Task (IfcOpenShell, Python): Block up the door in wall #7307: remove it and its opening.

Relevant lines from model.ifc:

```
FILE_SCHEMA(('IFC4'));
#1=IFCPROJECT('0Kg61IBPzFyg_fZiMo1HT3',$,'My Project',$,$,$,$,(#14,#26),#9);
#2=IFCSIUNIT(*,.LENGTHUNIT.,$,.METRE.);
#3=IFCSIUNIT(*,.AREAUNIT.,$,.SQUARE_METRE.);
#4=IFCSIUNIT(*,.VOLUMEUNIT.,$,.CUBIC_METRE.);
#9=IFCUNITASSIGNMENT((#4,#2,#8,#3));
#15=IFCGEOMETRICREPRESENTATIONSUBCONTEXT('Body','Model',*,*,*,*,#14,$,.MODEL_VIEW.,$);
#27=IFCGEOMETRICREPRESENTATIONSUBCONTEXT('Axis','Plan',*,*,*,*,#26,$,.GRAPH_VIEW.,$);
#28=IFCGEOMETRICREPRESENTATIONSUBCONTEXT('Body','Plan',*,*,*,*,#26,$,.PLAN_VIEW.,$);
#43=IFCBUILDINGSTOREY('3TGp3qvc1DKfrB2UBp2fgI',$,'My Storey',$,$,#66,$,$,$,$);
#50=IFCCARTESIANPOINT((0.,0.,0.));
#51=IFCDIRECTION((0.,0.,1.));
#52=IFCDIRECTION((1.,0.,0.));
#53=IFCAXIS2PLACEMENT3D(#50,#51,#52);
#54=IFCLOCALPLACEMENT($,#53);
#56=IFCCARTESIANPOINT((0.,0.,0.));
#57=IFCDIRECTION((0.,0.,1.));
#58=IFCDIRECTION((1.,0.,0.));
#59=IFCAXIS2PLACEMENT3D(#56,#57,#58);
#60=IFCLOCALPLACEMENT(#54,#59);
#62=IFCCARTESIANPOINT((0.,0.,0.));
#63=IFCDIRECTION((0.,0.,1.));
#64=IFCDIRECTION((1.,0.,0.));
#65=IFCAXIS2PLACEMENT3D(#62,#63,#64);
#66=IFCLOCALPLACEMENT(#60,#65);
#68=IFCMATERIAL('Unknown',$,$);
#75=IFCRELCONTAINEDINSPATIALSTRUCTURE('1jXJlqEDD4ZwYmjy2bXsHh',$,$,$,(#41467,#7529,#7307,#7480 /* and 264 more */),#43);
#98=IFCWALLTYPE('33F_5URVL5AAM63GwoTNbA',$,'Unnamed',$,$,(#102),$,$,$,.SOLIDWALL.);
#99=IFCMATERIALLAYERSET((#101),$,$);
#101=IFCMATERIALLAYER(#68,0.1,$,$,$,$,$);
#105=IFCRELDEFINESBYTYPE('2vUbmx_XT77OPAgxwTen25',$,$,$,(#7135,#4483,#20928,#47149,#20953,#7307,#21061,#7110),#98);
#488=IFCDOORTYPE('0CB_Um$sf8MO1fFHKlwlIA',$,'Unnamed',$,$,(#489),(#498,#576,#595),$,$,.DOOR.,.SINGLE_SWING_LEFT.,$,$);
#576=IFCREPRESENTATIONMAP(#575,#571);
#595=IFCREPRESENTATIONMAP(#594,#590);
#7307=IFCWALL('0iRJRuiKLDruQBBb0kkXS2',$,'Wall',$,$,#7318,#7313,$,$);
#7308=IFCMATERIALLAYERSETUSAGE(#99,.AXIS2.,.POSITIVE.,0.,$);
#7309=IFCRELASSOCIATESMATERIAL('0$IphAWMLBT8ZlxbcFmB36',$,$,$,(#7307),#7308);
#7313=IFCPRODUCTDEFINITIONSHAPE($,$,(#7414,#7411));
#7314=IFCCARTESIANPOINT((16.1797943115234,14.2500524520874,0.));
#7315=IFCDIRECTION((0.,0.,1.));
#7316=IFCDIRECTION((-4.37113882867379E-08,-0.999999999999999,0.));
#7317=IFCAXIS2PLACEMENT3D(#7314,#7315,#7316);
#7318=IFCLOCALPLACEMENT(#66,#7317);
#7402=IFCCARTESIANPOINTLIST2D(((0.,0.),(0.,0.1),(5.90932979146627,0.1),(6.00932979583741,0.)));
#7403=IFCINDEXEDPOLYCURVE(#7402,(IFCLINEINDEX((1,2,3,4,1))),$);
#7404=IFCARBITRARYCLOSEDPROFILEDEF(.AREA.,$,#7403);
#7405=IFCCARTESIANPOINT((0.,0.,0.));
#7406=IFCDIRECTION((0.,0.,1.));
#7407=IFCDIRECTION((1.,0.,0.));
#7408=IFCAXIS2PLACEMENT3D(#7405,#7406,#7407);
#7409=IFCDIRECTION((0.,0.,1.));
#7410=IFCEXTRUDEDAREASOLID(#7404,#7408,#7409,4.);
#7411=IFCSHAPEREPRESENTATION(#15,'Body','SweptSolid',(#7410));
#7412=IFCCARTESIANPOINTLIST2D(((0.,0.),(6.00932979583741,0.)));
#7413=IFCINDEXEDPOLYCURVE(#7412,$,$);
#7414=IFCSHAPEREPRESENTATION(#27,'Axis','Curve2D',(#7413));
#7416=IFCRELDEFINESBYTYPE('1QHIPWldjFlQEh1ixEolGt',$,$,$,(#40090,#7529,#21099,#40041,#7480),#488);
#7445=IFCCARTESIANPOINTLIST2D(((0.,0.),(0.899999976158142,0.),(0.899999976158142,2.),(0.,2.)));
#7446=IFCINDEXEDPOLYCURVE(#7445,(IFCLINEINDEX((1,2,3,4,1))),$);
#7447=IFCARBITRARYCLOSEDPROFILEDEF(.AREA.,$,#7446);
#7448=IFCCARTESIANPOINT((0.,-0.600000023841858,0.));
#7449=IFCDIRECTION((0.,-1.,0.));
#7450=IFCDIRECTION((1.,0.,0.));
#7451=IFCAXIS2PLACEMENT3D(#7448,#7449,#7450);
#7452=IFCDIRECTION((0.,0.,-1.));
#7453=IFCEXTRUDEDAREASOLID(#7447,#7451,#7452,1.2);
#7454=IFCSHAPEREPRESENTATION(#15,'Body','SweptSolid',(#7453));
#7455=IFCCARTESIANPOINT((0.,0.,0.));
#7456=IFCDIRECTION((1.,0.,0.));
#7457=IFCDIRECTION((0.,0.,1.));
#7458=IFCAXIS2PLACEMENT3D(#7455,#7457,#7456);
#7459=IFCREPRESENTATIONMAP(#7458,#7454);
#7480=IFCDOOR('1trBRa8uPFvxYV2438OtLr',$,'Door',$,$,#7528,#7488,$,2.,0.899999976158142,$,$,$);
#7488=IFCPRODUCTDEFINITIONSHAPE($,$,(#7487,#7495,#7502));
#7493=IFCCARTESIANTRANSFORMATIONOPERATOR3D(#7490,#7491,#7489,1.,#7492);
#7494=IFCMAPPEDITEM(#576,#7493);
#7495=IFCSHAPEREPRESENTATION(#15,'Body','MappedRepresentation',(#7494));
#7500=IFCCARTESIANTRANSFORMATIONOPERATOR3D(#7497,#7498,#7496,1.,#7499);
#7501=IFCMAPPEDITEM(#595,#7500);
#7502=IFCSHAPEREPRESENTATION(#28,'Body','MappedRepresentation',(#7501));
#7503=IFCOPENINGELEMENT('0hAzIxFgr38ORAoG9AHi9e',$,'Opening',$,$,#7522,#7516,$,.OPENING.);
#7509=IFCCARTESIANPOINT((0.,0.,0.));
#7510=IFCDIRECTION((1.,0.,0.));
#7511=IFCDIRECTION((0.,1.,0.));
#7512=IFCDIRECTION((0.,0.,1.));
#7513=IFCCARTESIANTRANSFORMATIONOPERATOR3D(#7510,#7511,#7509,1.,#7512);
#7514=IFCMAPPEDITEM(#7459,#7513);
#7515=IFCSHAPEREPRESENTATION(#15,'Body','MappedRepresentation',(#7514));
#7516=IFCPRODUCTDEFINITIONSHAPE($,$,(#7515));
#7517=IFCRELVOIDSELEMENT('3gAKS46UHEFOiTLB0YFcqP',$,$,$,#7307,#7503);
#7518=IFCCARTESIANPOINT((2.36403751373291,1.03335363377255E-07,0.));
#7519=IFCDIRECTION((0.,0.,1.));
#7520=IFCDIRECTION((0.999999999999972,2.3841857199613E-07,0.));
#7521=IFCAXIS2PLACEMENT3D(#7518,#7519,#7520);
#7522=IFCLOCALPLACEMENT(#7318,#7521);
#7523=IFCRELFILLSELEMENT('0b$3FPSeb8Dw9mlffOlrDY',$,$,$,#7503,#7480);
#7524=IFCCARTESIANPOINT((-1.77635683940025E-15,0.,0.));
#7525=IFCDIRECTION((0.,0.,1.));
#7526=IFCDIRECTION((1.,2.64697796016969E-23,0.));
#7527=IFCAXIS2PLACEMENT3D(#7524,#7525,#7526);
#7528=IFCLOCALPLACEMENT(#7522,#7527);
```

```python
import ifcopenshell
import ifcopenshell.api.feature
import ifcopenshell.api.root
import ifcopenshell.geom
import ifcopenshell.util.shape

model = ifcopenshell.open("model.ifc")
settings = ifcopenshell.geom.settings()


def volume(element):
    """Net volume in cubic metres, openings subtracted."""
    shape = ifcopenshell.geom.create_shape(settings, element)
    return ifcopenshell.util.shape.get_volume(shape.geometry)


door = model.by_guid("1trBRa8uPFvxYV2438OtLr")
opening = door.FillsVoids[0].RelatingOpeningElement
wall = opening.VoidsElements[0].RelatingBuildingElement
before = volume(wall)

ifcopenshell.api.root.remove_product(model, product=door)
ifcopenshell.api.feature.remove_feature(model, feature=opening)

after = volume(wall)

print(f"wall volume {before:.3f} -> {after:.3f} m3")

model.write("model_rev.ifc")
```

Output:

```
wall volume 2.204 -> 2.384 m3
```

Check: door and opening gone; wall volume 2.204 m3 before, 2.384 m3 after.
